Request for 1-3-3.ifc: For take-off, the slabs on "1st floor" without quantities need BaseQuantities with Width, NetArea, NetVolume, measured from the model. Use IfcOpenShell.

First a look at what the model holds.

```python
import ifcopenshell
import ifcopenshell.util.element
import ifcopenshell.util.unit

model = ifcopenshell.open("1-3-3.ifc")
print(model.schema)
for unit_type in ("LENGTHUNIT", "AREAUNIT", "VOLUMEUNIT"):
    print(unit_type, ifcopenshell.util.unit.calculate_unit_scale(model, unit_type))
storey = next(s for s in model.by_type("IfcBuildingStorey") if s.Name == "1st floor")
slabs = [e for e in ifcopenshell.util.element.get_decomposition(storey) if e.is_a("IfcSlab")]
for e in sorted(slabs, key=lambda e: e.id()):
    print(e.id(), e.is_a(), e.Name, list(ifcopenshell.util.element.get_psets(e, qtos_only=True)), sep=" | ")
```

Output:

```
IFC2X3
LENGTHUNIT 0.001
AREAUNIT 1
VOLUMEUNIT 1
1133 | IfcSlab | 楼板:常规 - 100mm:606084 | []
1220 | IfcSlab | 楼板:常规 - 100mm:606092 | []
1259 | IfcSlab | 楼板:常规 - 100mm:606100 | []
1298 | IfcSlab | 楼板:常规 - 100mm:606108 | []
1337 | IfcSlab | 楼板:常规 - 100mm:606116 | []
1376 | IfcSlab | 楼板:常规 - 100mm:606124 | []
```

```python
import ifcopenshell
import ifcopenshell.api.pset
import ifcopenshell.geom
import ifcopenshell.util.element
import ifcopenshell.util.shape
import ifcopenshell.util.unit

model = ifcopenshell.open("1-3-3.ifc")
unit_scale = ifcopenshell.util.unit.calculate_unit_scale(model)
area_scale = ifcopenshell.util.unit.calculate_unit_scale(model, "AREAUNIT")
volume_scale = ifcopenshell.util.unit.calculate_unit_scale(model, "VOLUMEUNIT")
settings = ifcopenshell.geom.settings()

storey = next(s for s in model.by_type("IfcBuildingStorey") if s.Name == "1st floor")
slabs = [e for e in ifcopenshell.util.element.get_decomposition(storey) if e.is_a("IfcSlab")]

for e in sorted(slabs, key=lambda e: e.id()):
    if ifcopenshell.util.element.get_psets(e, qtos_only=True, should_inherit=False):
        continue
    # Geometry comes back in metres, in the element's own axes.
    shape = ifcopenshell.geom.create_shape(settings, e)
    values = {
        "Width": ifcopenshell.util.shape.get_z(shape.geometry) / unit_scale,
        "NetArea": ifcopenshell.util.shape.get_footprint_area(shape.geometry) / area_scale,
        "NetVolume": ifcopenshell.util.shape.get_volume(shape.geometry) / volume_scale,
    }
    qto = ifcopenshell.api.pset.add_qto(model, product=e, name="BaseQuantities")
    ifcopenshell.api.pset.edit_qto(model, qto=qto, properties=values)
    print(e.id(), {k: round(v, 3) for k, v in values.items()})

model.write("1-3-3_v2.ifc")
```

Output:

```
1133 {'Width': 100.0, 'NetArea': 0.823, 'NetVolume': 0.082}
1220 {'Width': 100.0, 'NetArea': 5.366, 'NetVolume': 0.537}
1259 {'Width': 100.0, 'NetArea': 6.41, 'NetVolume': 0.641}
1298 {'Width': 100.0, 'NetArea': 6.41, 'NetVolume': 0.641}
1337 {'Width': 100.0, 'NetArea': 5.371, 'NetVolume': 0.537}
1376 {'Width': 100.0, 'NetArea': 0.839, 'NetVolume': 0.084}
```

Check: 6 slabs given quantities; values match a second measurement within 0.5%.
